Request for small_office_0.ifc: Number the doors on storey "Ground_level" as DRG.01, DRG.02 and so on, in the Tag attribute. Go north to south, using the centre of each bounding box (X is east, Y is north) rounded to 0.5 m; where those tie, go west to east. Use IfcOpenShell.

First a look at what the model holds.

```python
import ifcopenshell
import ifcopenshell.util.element
import ifcopenshell.util.placement

model = ifcopenshell.open("small_office_0.ifc")
print(model.schema)
storey = next(s for s in model.by_type("IfcBuildingStorey") if s.Name == "Ground_level")
doors = [e for e in ifcopenshell.util.element.get_decomposition(storey) if e.is_a("IfcDoor")]
for e in sorted(doors, key=lambda e: e.id()):
    origin = ifcopenshell.util.placement.get_local_placement(e.ObjectPlacement)[:3, 3]
    print(e.id(), e.Tag, e.Name, origin.round(2) + 0.0, sep=" | ")
```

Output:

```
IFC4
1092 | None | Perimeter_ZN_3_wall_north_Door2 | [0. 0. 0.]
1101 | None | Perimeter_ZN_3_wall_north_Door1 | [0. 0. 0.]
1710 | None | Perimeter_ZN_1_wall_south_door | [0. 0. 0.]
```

```python
import ifcopenshell
import ifcopenshell.geom
import ifcopenshell.util.element
import ifcopenshell.util.shape

model = ifcopenshell.open("small_office_0.ifc")
settings = ifcopenshell.geom.settings()
settings.set("use-world-coords", True)


def centre(element):
    shape = ifcopenshell.geom.create_shape(settings, element)
    return ifcopenshell.util.shape.get_bbox_centroid(shape.geometry)


storey = next(s for s in model.by_type("IfcBuildingStorey") if s.Name == "Ground_level")
doors = [e for e in ifcopenshell.util.element.get_decomposition(storey) if e.is_a("IfcDoor")]

# Insertion points can sit at a corner or the storey origin, so sort by the geometry (in metres).
centres = {e: centre(e) for e in doors}
doors.sort(key=lambda e: (-round(centres[e][1] / 0.5), centres[e][0]))

for i, e in enumerate(doors, start=1):
    number = f"DRG.{i:02d}"
    e.Tag = number
    print(e.id(), number)

model.write("small_office_0-out.ifc")
```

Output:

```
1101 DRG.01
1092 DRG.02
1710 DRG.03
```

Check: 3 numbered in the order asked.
